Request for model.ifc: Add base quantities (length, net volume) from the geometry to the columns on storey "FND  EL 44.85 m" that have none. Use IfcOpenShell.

First a look at what the model holds.

```python
import ifcopenshell
import ifcopenshell.util.element
import ifcopenshell.util.unit

model = ifcopenshell.open("model.ifc")
print(model.schema)
for unit_type in ("LENGTHUNIT", "AREAUNIT", "VOLUMEUNIT"):
    print(unit_type, ifcopenshell.util.unit.calculate_unit_scale(model, unit_type))
storey = next(s for s in model.by_type("IfcBuildingStorey") if s.Name == "FND  EL 44.85 m")
columns = [e for e in ifcopenshell.util.element.get_decomposition(storey) if e.is_a("IfcColumn")]
for e in sorted(columns, key=lambda e: e.id()):
    print(e.id(), e.is_a(), e.Name, list(ifcopenshell.util.element.get_psets(e, qtos_only=True)), sep=" | ")
```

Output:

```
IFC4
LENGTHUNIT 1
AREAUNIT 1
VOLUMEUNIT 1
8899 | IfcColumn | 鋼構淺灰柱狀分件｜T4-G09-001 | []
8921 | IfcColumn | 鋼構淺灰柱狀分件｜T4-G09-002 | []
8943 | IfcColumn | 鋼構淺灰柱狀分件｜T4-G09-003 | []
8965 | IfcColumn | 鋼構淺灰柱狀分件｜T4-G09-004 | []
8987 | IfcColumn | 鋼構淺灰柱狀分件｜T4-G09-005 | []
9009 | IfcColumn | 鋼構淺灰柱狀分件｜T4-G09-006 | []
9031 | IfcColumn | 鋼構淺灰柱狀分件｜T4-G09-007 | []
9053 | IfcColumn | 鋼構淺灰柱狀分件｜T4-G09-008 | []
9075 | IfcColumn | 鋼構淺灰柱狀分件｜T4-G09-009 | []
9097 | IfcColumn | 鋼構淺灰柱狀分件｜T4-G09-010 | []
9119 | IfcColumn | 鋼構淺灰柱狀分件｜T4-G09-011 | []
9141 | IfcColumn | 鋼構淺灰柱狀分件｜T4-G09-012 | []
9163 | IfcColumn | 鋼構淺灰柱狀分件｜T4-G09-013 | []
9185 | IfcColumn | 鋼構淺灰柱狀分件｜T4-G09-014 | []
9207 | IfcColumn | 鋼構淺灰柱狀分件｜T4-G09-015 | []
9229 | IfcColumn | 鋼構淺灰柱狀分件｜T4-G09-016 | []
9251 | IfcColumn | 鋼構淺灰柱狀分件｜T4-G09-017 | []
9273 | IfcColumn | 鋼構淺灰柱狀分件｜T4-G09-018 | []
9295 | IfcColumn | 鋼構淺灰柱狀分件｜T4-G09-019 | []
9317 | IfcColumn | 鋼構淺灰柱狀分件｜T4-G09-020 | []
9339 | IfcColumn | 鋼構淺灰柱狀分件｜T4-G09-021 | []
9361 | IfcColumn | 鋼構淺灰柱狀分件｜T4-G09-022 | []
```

```python
import ifcopenshell
import ifcopenshell.api.pset
import ifcopenshell.geom
import ifcopenshell.util.element
import ifcopenshell.util.shape
import ifcopenshell.util.unit

model = ifcopenshell.open("model.ifc")
unit_scale = ifcopenshell.util.unit.calculate_unit_scale(model)
volume_scale = ifcopenshell.util.unit.calculate_unit_scale(model, "VOLUMEUNIT")
settings = ifcopenshell.geom.settings()

storey = next(s for s in model.by_type("IfcBuildingStorey") if s.Name == "FND  EL 44.85 m")
columns = [e for e in ifcopenshell.util.element.get_decomposition(storey) if e.is_a("IfcColumn")]

for e in sorted(columns, key=lambda e: e.id()):
    if ifcopenshell.util.element.get_psets(e, qtos_only=True, should_inherit=False):
        continue
    # Geometry comes back in metres, in the element's own axes.
    shape = ifcopenshell.geom.create_shape(settings, e)
    values = {
        "Length": ifcopenshell.util.shape.get_z(shape.geometry) / unit_scale,
        "NetVolume": ifcopenshell.util.shape.get_volume(shape.geometry) / volume_scale,
    }
    qto = ifcopenshell.api.pset.add_qto(model, product=e, name="Qto_ColumnBaseQuantities")
    ifcopenshell.api.pset.edit_qto(model, qto=qto, properties=values)
    print(e.id(), {k: round(v, 3) for k, v in values.items()})

model.write("model-out.ifc")
```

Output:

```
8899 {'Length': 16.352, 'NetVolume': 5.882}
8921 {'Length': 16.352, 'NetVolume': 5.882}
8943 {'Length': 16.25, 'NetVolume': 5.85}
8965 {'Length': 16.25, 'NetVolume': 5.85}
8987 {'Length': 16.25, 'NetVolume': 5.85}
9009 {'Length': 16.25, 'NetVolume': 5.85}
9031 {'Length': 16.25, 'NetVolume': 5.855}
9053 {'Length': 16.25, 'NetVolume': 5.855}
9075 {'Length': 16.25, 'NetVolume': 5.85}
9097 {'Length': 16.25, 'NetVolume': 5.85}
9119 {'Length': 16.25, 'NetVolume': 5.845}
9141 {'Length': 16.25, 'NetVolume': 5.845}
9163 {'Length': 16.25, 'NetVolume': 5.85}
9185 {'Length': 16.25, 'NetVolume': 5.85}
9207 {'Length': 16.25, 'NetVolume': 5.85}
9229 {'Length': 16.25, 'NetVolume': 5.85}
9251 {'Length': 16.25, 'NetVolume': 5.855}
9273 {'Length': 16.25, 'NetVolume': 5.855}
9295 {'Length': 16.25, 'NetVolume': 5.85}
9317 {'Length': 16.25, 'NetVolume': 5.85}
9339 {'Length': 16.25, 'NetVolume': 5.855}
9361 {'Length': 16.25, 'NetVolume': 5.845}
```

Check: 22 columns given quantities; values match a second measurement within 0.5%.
